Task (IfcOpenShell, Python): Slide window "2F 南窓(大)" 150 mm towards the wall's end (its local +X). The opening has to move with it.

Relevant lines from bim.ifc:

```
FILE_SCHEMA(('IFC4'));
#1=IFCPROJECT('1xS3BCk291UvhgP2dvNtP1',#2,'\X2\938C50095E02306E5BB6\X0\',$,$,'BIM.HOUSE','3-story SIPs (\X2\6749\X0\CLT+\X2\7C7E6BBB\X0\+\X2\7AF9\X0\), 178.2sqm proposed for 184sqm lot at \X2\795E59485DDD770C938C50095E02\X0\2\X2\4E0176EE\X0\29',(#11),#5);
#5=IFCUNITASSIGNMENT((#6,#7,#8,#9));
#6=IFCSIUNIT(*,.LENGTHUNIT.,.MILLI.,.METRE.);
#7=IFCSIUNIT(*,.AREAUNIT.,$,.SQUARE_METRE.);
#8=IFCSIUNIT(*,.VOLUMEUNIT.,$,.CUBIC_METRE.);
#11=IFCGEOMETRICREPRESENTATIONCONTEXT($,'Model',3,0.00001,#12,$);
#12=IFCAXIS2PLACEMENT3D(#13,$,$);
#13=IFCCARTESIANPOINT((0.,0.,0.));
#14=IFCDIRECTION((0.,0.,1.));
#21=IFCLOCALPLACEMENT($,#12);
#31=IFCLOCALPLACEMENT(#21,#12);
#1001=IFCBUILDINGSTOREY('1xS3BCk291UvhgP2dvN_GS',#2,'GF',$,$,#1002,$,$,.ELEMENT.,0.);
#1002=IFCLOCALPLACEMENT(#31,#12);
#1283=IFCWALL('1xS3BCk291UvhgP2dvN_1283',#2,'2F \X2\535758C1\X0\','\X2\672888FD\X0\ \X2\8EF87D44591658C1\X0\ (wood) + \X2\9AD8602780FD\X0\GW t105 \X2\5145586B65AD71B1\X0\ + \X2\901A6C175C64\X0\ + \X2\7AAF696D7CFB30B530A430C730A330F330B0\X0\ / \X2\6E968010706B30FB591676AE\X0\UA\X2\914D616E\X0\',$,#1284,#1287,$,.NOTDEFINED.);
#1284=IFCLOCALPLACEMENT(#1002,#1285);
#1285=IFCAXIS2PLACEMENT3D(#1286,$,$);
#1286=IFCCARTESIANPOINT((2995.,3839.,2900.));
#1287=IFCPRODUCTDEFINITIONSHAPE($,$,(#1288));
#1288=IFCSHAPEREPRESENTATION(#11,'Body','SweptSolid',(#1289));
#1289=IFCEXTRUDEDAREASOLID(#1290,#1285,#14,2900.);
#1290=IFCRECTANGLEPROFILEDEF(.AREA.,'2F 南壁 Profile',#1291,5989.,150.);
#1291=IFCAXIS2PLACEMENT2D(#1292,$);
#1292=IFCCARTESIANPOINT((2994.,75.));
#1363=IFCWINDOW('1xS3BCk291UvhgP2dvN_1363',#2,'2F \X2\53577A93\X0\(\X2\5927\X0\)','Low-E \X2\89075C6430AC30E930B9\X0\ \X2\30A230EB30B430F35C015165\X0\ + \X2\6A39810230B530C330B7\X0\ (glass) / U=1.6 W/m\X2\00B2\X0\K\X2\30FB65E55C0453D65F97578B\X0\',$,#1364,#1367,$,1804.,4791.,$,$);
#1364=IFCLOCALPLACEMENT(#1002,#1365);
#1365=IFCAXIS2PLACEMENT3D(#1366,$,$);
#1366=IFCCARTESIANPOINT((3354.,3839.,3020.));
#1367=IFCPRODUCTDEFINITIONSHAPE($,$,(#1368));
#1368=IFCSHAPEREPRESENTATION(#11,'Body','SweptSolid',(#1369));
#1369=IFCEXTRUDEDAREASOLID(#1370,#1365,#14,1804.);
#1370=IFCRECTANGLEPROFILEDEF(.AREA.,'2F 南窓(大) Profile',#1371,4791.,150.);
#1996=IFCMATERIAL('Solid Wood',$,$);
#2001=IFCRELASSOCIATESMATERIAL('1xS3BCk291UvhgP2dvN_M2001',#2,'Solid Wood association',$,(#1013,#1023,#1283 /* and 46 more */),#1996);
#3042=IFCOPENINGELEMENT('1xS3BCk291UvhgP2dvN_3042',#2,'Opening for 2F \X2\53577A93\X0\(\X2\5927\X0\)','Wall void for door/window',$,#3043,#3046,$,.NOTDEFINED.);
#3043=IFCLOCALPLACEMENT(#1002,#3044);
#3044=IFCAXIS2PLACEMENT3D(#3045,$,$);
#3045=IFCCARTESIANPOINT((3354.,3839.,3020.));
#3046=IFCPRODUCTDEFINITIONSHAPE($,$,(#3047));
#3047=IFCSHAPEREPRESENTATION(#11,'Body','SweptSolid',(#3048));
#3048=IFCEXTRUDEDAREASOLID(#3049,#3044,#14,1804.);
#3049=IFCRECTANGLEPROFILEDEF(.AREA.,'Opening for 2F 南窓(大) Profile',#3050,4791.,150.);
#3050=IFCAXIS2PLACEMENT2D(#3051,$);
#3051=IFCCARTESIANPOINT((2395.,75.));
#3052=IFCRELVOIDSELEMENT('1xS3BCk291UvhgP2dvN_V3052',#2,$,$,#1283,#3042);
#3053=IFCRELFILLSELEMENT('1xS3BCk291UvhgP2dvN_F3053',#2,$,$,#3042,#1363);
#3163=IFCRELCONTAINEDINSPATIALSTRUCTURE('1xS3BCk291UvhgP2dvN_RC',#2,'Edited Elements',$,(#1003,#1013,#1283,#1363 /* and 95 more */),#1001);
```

```python
import ifcopenshell
import ifcopenshell.api.geometry
import ifcopenshell.util.placement
import ifcopenshell.util.unit

model = ifcopenshell.open("bim.ifc")
unit_scale = ifcopenshell.util.unit.calculate_unit_scale(model)

window = model.by_id(1363)
opening = window.FillsVoids[0].RelatingOpeningElement
wall = opening.VoidsElements[0].RelatingBuildingElement

wall_matrix = ifcopenshell.util.placement.get_local_placement(wall.ObjectPlacement)
shift = wall_matrix[:3, 0] * 0.15 / unit_scale
before = ifcopenshell.util.placement.get_local_placement(window.ObjectPlacement)[:3, 3].copy()

# The window is not placed relative to its opening, so move both.
for product in (opening, window):
    matrix = ifcopenshell.util.placement.get_local_placement(product.ObjectPlacement)
    matrix[:3, 3] += shift
    ifcopenshell.api.geometry.edit_object_placement(model, product=product, matrix=matrix, is_si=False)

after = ifcopenshell.util.placement.get_local_placement(window.ObjectPlacement)[:3, 3]
print("window moved by", (after - before).round(3) + 0.0)

model.write("bim_rev.ifc")
```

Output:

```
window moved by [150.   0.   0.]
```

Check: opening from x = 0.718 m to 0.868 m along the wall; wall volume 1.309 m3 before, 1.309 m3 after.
